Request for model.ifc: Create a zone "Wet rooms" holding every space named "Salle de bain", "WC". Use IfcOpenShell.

First a look at what the model holds.

```python
import ifcopenshell

model = ifcopenshell.open("model.ifc")
print(model.schema)
seen = {}
for space in model.by_type("IfcSpace"):
    seen[space.LongName] = seen.get(space.LongName, 0) + 1
for name, count in sorted(seen.items(), key=str):
    print(count, "x", name)
print("zones:", [z.Name for z in model.by_type("IfcZone")][:20])
```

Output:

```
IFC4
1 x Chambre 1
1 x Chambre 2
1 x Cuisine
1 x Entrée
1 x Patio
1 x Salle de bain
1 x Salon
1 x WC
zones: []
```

```python
import ifcopenshell
import ifcopenshell.api.group
import ifcopenshell.api.root

model = ifcopenshell.open("model.ifc")

names = {"Salle de bain", "WC"}
spaces = [s for s in model.by_type("IfcSpace") if s.LongName in names]

zone = ifcopenshell.api.root.create_entity(model, ifc_class="IfcZone", name="Wet rooms")
ifcopenshell.api.group.assign_group(model, products=spaces, group=zone)
print(len(spaces), "spaces in", zone.Name)

model.write("model_rev.ifc")
```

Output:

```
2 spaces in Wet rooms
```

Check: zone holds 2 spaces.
